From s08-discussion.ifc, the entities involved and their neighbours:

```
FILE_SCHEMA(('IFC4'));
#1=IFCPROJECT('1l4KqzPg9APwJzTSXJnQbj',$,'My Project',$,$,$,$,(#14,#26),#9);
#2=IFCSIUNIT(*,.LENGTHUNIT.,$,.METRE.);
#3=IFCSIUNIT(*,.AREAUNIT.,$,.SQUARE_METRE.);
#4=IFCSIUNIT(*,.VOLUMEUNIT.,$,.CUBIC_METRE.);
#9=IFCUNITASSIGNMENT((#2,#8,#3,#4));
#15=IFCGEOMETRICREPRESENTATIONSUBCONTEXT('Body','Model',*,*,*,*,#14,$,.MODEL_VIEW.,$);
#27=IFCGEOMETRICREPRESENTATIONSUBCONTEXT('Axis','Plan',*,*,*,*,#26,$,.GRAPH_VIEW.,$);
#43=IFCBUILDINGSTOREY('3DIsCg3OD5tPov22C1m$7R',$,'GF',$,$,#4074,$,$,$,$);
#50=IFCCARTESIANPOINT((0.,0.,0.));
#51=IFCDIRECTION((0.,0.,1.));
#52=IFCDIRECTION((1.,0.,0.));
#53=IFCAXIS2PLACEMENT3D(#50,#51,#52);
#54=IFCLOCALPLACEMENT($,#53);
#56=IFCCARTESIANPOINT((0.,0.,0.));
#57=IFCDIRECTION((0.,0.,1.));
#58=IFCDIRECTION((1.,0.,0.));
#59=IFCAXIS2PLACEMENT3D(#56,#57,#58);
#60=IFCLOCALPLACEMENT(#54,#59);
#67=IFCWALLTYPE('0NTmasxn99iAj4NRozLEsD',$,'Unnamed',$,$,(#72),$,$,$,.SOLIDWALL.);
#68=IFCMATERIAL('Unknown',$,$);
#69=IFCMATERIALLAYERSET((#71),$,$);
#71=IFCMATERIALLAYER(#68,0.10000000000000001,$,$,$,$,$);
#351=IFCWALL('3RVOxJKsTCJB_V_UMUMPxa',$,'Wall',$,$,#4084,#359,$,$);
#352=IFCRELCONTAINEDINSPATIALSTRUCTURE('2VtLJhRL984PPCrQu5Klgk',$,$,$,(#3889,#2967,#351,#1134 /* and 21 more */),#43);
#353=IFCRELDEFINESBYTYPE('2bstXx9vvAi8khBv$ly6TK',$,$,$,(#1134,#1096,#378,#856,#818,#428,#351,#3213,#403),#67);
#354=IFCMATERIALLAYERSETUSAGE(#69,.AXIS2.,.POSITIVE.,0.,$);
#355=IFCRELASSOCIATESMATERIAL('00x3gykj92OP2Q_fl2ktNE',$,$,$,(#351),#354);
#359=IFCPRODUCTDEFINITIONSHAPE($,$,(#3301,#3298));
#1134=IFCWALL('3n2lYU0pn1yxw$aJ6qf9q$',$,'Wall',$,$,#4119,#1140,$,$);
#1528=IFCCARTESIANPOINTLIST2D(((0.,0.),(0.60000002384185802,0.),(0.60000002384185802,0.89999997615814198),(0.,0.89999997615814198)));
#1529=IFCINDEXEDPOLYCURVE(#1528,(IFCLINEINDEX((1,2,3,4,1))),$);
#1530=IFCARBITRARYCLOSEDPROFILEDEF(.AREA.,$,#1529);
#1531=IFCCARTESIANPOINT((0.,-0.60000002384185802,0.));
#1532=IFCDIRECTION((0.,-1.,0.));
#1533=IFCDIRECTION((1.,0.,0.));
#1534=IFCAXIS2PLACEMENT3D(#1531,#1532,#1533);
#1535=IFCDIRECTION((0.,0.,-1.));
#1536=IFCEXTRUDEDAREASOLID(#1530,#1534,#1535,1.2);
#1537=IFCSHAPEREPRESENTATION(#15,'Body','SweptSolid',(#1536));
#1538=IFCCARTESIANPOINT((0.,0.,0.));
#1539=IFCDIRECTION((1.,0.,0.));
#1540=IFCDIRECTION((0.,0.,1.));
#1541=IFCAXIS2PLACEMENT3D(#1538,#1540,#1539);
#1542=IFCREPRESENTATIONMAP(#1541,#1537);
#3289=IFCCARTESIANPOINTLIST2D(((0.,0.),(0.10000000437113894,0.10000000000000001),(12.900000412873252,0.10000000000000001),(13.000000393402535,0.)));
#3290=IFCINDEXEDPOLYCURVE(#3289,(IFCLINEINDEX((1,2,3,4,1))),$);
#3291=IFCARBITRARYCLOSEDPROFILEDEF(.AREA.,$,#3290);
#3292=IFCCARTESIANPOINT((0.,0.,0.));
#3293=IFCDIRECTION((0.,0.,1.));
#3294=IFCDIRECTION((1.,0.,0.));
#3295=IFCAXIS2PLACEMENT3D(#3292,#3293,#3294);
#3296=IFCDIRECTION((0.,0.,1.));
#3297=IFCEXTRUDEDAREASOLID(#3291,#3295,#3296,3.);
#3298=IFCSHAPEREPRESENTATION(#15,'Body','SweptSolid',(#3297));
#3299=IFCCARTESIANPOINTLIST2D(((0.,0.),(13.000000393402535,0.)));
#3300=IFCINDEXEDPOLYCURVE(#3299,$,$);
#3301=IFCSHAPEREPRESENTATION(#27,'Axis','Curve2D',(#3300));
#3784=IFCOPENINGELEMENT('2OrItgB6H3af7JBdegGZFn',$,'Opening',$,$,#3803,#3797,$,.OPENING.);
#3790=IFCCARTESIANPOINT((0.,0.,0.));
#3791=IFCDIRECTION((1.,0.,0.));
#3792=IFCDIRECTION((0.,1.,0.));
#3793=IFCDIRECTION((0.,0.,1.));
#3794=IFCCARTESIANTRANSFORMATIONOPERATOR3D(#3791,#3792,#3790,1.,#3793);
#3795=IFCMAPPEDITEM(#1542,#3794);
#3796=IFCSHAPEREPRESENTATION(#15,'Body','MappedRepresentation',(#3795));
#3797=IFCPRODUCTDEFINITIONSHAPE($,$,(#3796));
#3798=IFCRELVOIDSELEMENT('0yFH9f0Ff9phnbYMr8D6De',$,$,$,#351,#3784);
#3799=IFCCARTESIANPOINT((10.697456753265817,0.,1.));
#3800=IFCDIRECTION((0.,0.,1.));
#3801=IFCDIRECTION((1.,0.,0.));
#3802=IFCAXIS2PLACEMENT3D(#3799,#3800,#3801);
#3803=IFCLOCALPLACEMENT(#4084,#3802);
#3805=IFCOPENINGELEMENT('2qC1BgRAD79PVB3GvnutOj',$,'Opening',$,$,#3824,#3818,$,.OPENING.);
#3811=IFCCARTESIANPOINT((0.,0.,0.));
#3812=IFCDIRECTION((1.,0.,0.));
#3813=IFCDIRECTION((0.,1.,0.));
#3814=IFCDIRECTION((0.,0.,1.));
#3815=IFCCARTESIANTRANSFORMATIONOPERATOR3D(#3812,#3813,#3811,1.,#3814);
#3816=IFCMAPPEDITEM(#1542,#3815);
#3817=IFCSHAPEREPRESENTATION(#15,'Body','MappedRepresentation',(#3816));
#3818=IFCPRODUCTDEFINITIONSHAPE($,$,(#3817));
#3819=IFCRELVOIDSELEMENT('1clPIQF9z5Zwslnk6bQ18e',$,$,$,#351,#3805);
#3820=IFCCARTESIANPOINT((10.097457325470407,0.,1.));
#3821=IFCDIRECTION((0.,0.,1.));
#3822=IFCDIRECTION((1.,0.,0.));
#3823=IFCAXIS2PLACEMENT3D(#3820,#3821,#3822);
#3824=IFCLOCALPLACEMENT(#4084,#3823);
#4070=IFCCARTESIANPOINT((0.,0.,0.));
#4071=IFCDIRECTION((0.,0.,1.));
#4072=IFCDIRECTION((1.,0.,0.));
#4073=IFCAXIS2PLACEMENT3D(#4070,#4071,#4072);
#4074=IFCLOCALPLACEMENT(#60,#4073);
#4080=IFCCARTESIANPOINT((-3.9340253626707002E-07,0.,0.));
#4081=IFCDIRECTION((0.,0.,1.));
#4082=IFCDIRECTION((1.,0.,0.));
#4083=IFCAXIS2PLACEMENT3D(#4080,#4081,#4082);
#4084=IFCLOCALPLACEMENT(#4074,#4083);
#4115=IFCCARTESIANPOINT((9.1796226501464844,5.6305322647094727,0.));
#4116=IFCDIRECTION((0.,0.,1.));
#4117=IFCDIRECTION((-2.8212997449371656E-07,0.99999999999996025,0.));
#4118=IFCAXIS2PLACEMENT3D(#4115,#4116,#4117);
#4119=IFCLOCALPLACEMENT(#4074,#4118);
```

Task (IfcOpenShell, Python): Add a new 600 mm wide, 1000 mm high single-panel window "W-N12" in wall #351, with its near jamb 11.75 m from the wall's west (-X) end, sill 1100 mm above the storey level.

```python
import numpy as np
import ifcopenshell
import ifcopenshell.api.feature
import ifcopenshell.api.geometry
import ifcopenshell.api.root
import ifcopenshell.api.spatial
import ifcopenshell.geom
import ifcopenshell.util.element
import ifcopenshell.util.placement
import ifcopenshell.util.representation
import ifcopenshell.util.shape
import ifcopenshell.util.unit

model = ifcopenshell.open("s08-discussion.ifc")
unit_scale = ifcopenshell.util.unit.calculate_unit_scale(model)
settings = ifcopenshell.geom.settings()


def volume(element):
    """Net volume in cubic metres, openings subtracted."""
    shape = ifcopenshell.geom.create_shape(settings, element)
    return ifcopenshell.util.shape.get_volume(shape.geometry)


wall = model.by_id(351)
storey = ifcopenshell.util.element.get_container(wall, ifc_class="IfcBuildingStorey")
context = ifcopenshell.util.representation.get_context(model, "Model", "Body", "MODEL_VIEW")
before = volume(wall)

width, height, from_end, sill = 0.6, 1, 11.75, 1.1  # metres

# The wall runs along its own X axis, and the end named is its -X end.
wall_shape = ifcopenshell.geom.create_shape(settings, wall)
x, y, z = ifcopenshell.util.shape.get_vertices(wall_shape.geometry).T
start = x.min() + from_end
face, thickness = float(y.min()), float(y.max() - y.min())
wall_matrix = ifcopenshell.util.placement.get_local_placement(wall.ObjectPlacement)
level = ifcopenshell.util.placement.get_local_placement(storey.ObjectPlacement)[2, 3]


def in_wall(x, y):
    """Placement at x, y metres in the wall's axes, at sill height."""
    matrix = wall_matrix.copy()
    matrix[:, 3] = wall_matrix @ np.array([x / unit_scale, y / unit_scale, 0.0, 1.0])
    matrix[2, 3] = level + sill / unit_scale
    return matrix


# Opening: a box that overshoots both wall faces by 50 mm.
opening = ifcopenshell.api.root.create_entity(model, ifc_class="IfcOpeningElement", predefined_type="OPENING")
box = ifcopenshell.api.geometry.add_wall_representation(
    model, context=context, length=width, height=height, thickness=thickness + 0.1
)
ifcopenshell.api.geometry.assign_representation(model, product=opening, representation=box)
ifcopenshell.api.geometry.edit_object_placement(model, product=opening, matrix=in_wall(start, face - 0.05), is_si=False)
ifcopenshell.api.feature.add_feature(model, feature=opening, element=wall)

window = ifcopenshell.api.root.create_entity(model, ifc_class="IfcWindow", name="W-N12", predefined_type="WINDOW")
window.OverallWidth, window.OverallHeight = width / unit_scale, height / unit_scale
window.PartitioningType = "SINGLE_PANEL"
body = ifcopenshell.api.geometry.add_window_representation(
    model,
    context=context,
    overall_width=window.OverallWidth,
    overall_height=window.OverallHeight,
    partition_type="SINGLE_PANEL",
)
ifcopenshell.api.geometry.assign_representation(model, product=window, representation=body)
ifcopenshell.api.spatial.assign_container(model, products=[window], relating_structure=storey)
ifcopenshell.api.feature.add_filling(model, opening=opening, element=window)

# Centre the window in the wall's thickness.
ifcopenshell.api.geometry.edit_object_placement(model, product=window, matrix=in_wall(start, face), is_si=False)
window_shape = ifcopenshell.geom.create_shape(settings, window)
depth = ifcopenshell.util.shape.get_vertices(window_shape.geometry)[:, 1]
offset = face + thickness / 2 - (depth.min() + depth.max()) / 2
ifcopenshell.api.geometry.edit_object_placement(model, product=window, matrix=in_wall(start, offset), is_si=False)

after = volume(wall)

print(f"wall volume {before:.3f} -> {after:.3f} m3")

model.write("s08-discussion_edited.ifc")
```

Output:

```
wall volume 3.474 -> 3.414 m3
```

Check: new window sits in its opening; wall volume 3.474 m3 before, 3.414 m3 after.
